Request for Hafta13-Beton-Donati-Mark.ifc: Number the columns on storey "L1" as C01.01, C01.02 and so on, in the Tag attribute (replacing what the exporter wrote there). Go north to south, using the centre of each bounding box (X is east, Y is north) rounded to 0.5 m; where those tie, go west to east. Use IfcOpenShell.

First a look at what the model holds.

```python
import ifcopenshell
import ifcopenshell.util.element
import ifcopenshell.util.placement

model = ifcopenshell.open("Hafta13-Beton-Donati-Mark.ifc")
print(model.schema)
storey = next(s for s in model.by_type("IfcBuildingStorey") if s.Name == "L1")
columns = [e for e in ifcopenshell.util.element.get_decomposition(storey) if e.is_a("IfcColumn")]
for e in sorted(columns, key=lambda e: e.id()):
    origin = ifcopenshell.util.placement.get_local_placement(e.ObjectPlacement)[:3, 3]
    print(e.id(), e.Tag, e.Name, origin.round(2) + 0.0, sep=" | ")
```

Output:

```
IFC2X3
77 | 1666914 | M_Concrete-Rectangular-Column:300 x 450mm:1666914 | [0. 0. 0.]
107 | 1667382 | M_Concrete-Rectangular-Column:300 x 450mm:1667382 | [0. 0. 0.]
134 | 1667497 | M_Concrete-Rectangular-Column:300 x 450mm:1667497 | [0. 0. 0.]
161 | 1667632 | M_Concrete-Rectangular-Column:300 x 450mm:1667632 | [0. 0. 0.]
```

```python
import ifcopenshell
import ifcopenshell.geom
import ifcopenshell.util.element
import ifcopenshell.util.shape

model = ifcopenshell.open("Hafta13-Beton-Donati-Mark.ifc")
settings = ifcopenshell.geom.settings()
settings.set("use-world-coords", True)


def centre(element):
    shape = ifcopenshell.geom.create_shape(settings, element)
    return ifcopenshell.util.shape.get_bbox_centroid(shape.geometry)


storey = next(s for s in model.by_type("IfcBuildingStorey") if s.Name == "L1")
columns = [e for e in ifcopenshell.util.element.get_decomposition(storey) if e.is_a("IfcColumn")]

# Insertion points can sit at a corner or the storey origin, so sort by the geometry (in metres).
centres = {e: centre(e) for e in columns}
columns.sort(key=lambda e: (-round(centres[e][1] / 0.5), centres[e][0]))

for i, e in enumerate(columns, start=1):
    number = f"C01.{i:02d}"
    e.Tag = number
    print(e.id(), number)

model.write("Hafta13-Beton-Donati-Mark-out.ifc")
```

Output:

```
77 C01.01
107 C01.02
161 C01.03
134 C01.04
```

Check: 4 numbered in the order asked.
